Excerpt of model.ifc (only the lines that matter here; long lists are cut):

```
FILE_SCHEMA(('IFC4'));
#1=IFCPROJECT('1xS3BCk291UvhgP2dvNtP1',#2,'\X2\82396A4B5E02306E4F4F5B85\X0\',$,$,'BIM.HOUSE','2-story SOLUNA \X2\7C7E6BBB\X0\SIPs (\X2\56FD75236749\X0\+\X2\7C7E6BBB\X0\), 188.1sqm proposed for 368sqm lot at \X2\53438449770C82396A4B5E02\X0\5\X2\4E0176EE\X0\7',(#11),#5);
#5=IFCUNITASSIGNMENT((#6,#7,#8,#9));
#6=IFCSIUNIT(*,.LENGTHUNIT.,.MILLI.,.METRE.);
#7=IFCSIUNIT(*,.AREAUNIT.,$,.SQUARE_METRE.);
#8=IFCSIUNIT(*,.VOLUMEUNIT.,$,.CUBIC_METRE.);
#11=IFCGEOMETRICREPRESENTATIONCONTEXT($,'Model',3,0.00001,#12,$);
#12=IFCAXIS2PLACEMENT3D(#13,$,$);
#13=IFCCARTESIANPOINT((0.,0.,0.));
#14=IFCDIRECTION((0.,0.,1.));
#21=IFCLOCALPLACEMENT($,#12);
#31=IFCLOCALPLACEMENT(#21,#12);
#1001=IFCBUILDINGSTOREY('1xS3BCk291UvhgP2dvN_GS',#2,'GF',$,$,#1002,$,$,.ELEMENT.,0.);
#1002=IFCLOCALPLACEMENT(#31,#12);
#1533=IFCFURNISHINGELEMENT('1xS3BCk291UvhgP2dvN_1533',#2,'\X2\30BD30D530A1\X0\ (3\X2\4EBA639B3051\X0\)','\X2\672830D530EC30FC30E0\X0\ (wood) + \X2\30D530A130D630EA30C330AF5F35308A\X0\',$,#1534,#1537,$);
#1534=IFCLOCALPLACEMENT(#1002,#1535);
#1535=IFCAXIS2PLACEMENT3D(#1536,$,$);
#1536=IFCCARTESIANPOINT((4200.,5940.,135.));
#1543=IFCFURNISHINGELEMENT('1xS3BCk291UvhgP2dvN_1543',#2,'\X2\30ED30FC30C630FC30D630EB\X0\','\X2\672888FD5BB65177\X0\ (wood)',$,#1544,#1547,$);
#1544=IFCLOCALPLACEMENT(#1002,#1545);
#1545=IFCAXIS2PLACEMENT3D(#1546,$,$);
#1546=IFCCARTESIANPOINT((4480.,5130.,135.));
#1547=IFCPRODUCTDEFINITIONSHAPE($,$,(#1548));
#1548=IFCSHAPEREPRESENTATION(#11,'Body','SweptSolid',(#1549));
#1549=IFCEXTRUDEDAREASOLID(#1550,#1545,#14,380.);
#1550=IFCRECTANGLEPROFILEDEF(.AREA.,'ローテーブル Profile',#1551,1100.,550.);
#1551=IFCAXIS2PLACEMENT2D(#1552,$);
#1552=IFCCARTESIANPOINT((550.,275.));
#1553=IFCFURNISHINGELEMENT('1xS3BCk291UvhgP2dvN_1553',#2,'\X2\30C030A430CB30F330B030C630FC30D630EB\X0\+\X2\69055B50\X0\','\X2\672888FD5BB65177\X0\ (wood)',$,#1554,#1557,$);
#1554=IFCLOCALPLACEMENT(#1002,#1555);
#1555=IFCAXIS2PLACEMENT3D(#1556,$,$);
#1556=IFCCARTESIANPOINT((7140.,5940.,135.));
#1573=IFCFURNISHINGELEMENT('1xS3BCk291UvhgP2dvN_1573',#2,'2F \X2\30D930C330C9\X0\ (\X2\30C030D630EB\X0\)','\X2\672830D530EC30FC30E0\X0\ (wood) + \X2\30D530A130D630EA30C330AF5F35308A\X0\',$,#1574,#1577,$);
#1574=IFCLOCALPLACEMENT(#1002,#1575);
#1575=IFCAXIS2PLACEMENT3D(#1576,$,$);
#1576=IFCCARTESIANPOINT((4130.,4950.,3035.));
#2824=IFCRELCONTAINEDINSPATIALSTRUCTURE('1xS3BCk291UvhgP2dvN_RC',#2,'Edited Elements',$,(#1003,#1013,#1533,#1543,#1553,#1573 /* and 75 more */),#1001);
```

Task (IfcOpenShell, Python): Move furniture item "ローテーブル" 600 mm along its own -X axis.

```python
import ifcopenshell
import ifcopenshell.api.geometry
import ifcopenshell.util.placement
import ifcopenshell.util.unit

model = ifcopenshell.open("model.ifc")
unit_scale = ifcopenshell.util.unit.calculate_unit_scale(model)

item = model.by_id(1543)
matrix = ifcopenshell.util.placement.get_local_placement(item.ObjectPlacement)
matrix[:3, 3] -= matrix[:3, 0] * 0.6 / unit_scale
ifcopenshell.api.geometry.edit_object_placement(model, product=item, matrix=matrix, is_si=False)

print(ifcopenshell.util.placement.get_local_placement(item.ObjectPlacement).round(3) + 0.0)

model.write("model_updated.ifc")
```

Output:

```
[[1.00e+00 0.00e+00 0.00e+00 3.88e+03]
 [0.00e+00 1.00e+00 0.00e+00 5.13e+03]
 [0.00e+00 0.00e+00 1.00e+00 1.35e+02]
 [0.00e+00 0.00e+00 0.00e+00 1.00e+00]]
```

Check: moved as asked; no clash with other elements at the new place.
